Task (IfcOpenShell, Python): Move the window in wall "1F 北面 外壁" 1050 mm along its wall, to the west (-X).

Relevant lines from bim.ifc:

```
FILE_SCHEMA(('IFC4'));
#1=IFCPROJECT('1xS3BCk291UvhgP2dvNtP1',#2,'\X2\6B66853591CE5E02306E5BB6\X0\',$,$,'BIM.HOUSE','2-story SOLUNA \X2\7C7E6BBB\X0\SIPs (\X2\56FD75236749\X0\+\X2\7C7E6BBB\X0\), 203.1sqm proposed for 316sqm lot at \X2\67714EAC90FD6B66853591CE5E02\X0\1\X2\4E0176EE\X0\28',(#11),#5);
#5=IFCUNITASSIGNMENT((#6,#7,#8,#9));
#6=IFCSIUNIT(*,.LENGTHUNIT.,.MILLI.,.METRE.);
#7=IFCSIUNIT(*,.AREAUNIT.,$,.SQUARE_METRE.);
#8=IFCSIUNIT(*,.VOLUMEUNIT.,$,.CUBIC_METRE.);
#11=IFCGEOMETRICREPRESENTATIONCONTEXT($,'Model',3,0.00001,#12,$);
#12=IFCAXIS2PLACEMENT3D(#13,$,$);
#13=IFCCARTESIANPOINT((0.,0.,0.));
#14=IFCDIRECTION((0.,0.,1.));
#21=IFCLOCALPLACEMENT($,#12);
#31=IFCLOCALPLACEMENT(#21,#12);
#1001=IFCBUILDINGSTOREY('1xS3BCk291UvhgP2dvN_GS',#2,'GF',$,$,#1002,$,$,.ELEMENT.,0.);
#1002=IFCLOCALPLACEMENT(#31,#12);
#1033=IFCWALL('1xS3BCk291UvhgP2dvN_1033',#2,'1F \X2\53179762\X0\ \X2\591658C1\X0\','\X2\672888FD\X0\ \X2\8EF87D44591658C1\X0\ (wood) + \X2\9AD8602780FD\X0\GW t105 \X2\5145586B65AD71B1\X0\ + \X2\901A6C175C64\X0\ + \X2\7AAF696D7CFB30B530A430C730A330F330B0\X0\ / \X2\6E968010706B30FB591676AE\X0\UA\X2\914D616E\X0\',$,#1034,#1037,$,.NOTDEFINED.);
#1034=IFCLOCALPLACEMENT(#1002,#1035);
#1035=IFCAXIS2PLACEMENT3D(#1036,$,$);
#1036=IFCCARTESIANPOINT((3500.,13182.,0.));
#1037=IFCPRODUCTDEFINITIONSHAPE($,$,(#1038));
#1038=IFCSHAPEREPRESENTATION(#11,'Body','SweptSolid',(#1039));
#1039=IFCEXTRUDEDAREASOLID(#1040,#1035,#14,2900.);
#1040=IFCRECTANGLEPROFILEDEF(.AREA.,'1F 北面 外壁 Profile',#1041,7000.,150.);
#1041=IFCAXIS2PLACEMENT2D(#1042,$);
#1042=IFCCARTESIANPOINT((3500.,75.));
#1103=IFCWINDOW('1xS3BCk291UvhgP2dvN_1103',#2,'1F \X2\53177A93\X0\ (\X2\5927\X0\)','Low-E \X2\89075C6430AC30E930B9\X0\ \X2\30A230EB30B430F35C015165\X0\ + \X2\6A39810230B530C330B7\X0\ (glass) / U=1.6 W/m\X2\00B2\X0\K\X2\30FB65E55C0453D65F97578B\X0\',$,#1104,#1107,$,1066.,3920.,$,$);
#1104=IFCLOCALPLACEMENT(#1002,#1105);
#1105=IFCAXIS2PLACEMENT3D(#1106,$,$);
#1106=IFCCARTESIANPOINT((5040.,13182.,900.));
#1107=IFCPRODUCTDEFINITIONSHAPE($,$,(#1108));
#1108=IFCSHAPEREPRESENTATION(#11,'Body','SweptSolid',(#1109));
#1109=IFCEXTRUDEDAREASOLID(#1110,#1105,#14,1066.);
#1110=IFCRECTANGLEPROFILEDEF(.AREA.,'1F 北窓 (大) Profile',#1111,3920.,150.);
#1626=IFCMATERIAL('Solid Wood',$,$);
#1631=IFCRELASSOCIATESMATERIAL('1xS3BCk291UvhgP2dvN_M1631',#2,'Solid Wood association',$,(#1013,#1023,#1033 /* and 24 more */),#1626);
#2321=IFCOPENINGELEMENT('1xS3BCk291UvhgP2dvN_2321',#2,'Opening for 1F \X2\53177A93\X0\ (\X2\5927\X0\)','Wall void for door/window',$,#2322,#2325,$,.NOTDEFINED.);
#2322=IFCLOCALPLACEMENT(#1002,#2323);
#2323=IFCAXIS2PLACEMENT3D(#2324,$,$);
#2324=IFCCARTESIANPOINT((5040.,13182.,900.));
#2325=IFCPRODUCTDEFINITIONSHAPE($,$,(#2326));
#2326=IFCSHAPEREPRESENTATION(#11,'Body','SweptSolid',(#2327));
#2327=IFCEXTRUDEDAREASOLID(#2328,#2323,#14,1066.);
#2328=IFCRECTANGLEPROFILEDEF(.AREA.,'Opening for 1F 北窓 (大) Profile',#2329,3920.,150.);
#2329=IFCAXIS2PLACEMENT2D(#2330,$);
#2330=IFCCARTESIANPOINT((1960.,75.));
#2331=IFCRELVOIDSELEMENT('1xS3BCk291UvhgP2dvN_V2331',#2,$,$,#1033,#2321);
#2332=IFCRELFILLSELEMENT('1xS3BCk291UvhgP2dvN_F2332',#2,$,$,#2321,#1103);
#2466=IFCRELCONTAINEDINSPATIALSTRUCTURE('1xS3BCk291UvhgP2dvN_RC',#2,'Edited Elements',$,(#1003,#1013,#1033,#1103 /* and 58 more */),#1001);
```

```python
import ifcopenshell
import ifcopenshell.api.geometry
import ifcopenshell.util.placement
import ifcopenshell.util.unit

model = ifcopenshell.open("bim.ifc")
unit_scale = ifcopenshell.util.unit.calculate_unit_scale(model)

window = model.by_id(1103)
opening = window.FillsVoids[0].RelatingOpeningElement
wall = opening.VoidsElements[0].RelatingBuildingElement

wall_matrix = ifcopenshell.util.placement.get_local_placement(wall.ObjectPlacement)
shift = wall_matrix[:3, 0] * -1.05 / unit_scale
before = ifcopenshell.util.placement.get_local_placement(window.ObjectPlacement)[:3, 3].copy()

# The window is not placed relative to its opening, so move both.
for product in (opening, window):
    matrix = ifcopenshell.util.placement.get_local_placement(product.ObjectPlacement)
    matrix[:3, 3] += shift
    ifcopenshell.api.geometry.edit_object_placement(model, product=product, matrix=matrix, is_si=False)

after = ifcopenshell.util.placement.get_local_placement(window.ObjectPlacement)[:3, 3]
print("window moved by", (after - before).round(3) + 0.0)

model.write("bim_rev.ifc")
```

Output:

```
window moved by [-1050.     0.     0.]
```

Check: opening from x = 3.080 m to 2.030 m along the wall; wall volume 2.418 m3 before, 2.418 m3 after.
